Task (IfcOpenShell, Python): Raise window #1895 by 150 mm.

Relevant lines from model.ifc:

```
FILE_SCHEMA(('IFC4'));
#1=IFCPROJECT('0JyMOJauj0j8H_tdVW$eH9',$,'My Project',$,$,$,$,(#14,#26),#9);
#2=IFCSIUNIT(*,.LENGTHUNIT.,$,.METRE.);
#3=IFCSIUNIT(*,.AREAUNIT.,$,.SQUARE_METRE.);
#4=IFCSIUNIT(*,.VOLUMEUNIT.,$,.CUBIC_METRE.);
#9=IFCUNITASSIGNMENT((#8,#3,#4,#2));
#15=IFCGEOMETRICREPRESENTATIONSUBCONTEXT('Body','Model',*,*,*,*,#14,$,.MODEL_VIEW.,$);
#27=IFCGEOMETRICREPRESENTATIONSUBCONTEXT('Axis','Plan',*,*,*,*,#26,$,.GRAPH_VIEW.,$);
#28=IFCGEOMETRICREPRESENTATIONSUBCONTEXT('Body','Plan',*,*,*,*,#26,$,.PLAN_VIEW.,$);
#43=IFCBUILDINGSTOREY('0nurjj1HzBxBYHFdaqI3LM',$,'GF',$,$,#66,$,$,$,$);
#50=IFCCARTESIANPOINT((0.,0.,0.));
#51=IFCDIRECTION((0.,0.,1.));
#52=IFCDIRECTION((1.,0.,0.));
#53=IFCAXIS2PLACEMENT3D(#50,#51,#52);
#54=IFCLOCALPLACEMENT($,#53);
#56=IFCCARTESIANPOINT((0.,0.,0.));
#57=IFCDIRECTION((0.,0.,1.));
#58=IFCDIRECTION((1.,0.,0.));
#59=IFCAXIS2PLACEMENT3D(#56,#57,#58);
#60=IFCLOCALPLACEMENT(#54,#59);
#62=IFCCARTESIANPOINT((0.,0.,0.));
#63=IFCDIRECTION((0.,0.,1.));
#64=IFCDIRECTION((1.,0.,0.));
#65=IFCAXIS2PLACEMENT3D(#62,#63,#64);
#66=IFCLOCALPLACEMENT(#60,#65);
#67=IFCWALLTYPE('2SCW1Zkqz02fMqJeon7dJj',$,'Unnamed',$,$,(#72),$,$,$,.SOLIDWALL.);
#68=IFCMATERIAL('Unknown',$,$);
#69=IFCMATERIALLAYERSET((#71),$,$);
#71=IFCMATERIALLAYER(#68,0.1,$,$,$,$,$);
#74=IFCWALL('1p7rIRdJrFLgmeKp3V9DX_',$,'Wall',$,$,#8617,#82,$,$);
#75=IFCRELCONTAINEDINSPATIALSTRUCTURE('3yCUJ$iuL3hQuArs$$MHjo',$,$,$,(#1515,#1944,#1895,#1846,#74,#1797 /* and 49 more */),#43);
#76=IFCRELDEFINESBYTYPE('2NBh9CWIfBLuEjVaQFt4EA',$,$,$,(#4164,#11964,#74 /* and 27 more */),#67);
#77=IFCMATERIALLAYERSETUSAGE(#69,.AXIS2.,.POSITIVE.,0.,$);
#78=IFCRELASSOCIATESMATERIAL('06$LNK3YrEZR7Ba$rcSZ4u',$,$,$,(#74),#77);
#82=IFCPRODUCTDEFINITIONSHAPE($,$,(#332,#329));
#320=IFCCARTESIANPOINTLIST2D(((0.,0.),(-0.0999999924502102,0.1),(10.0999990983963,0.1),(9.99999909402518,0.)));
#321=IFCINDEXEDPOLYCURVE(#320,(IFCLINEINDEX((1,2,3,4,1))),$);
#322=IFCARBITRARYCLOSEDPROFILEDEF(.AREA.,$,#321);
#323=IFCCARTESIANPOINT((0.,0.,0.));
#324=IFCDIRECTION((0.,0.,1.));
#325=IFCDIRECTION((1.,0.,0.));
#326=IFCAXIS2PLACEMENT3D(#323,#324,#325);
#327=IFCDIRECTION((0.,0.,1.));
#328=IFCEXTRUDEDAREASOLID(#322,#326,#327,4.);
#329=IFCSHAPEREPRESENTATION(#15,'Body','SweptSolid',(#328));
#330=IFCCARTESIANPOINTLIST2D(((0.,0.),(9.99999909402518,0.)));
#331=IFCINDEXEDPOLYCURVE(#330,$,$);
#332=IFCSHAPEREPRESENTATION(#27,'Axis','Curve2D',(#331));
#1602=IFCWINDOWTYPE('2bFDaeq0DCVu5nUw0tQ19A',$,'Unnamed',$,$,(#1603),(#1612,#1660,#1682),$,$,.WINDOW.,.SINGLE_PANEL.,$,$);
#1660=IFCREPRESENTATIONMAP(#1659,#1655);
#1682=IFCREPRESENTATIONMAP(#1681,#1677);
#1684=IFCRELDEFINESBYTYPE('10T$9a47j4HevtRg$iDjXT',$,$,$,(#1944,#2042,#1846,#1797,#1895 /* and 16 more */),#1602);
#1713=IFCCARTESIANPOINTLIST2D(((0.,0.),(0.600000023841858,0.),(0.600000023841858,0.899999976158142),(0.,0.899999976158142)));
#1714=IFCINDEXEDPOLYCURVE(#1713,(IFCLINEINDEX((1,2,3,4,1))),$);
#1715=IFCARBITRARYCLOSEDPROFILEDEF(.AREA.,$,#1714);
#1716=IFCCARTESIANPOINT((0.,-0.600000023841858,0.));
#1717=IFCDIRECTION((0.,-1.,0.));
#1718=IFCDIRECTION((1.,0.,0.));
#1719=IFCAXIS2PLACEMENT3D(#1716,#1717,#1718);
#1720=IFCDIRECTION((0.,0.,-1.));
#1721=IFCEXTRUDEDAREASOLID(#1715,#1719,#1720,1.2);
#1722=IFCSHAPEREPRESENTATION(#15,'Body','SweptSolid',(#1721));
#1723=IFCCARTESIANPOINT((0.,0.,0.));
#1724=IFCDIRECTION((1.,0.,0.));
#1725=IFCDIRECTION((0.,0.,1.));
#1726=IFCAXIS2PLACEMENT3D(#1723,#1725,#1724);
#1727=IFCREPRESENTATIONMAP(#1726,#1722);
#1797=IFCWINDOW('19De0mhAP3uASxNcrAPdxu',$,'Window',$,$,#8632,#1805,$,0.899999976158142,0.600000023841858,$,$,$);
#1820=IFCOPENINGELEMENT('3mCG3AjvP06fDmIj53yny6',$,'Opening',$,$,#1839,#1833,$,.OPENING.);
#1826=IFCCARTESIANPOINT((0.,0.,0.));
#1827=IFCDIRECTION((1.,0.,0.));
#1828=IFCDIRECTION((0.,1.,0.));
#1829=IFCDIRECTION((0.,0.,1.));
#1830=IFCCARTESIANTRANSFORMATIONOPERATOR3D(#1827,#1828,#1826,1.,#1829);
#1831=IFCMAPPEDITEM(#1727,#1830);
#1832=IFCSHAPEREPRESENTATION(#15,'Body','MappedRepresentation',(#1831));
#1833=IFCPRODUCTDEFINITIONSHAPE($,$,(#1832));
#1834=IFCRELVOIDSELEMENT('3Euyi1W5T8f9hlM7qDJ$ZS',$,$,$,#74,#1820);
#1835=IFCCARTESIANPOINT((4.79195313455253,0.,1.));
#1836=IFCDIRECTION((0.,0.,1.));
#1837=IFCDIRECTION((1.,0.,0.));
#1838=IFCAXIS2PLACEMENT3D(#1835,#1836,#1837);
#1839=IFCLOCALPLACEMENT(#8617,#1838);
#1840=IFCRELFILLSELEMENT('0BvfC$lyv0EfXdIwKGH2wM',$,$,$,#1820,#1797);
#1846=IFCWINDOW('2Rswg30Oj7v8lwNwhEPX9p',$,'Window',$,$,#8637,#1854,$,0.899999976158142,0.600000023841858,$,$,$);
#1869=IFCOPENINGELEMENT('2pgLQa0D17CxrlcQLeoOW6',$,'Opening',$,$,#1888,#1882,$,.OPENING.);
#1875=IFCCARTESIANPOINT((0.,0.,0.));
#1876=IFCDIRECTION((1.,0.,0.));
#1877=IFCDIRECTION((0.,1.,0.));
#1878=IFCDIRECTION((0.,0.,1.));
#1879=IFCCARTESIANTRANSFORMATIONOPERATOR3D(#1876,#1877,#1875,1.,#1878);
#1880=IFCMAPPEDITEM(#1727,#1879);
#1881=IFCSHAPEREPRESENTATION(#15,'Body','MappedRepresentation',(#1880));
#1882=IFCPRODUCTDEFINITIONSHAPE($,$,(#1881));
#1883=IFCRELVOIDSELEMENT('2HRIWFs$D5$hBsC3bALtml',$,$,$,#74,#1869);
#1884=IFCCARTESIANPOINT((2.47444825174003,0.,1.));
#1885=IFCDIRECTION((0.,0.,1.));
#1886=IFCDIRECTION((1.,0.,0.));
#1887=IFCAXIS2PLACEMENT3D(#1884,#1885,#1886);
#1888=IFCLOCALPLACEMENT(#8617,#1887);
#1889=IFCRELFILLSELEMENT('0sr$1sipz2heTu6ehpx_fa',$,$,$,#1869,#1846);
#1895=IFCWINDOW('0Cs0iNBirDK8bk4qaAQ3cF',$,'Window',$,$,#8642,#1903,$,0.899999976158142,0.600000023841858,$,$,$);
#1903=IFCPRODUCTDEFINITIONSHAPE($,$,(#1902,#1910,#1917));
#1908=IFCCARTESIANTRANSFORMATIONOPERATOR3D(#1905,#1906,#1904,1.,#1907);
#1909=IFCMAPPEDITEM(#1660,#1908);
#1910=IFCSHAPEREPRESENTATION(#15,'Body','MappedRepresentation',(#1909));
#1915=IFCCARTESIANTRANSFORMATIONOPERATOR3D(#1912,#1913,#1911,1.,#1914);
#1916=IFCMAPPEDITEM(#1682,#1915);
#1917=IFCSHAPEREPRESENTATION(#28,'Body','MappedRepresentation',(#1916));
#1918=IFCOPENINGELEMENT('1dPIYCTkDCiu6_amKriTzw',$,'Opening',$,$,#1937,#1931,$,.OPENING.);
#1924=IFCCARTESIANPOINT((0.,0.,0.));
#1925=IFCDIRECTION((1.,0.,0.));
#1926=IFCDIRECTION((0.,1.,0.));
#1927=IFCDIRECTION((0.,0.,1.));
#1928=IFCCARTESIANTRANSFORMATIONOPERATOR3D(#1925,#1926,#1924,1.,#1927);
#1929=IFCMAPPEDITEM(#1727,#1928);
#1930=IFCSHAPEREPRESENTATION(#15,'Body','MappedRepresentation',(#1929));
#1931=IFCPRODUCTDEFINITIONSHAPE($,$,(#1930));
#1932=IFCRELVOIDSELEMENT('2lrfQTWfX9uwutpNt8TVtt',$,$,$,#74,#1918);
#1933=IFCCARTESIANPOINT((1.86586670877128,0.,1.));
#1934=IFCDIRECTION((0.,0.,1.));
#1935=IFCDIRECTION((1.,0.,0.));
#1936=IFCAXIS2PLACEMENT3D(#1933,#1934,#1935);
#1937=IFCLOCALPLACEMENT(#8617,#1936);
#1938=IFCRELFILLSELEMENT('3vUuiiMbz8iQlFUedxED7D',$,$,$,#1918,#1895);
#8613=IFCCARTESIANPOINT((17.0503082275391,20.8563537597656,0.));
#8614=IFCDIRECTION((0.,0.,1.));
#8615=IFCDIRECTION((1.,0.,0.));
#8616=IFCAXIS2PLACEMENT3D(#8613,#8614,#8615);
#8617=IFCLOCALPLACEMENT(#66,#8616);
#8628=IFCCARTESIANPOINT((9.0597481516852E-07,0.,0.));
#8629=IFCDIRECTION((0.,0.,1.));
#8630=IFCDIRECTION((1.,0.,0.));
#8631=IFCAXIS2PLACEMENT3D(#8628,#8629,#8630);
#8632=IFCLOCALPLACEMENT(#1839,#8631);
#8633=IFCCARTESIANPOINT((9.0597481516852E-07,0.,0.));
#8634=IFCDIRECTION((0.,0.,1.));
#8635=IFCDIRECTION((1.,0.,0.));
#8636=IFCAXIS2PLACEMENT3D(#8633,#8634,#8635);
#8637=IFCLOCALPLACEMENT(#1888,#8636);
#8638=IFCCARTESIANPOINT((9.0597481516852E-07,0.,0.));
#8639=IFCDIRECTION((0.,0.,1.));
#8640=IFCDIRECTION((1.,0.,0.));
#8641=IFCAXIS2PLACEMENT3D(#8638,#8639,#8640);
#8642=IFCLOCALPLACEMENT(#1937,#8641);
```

```python
import numpy as np
import ifcopenshell
import ifcopenshell.api.geometry
import ifcopenshell.util.placement
import ifcopenshell.util.unit

model = ifcopenshell.open("model.ifc")
unit_scale = ifcopenshell.util.unit.calculate_unit_scale(model)

window = model.by_guid("0Cs0iNBirDK8bk4qaAQ3cF")
opening = window.FillsVoids[0].RelatingOpeningElement
dz = 0.15 / unit_scale

shift = np.array([0.0, 0.0, dz])
# The window is placed relative to its opening, so it follows when the opening moves.
matrix = ifcopenshell.util.placement.get_local_placement(opening.ObjectPlacement)
matrix[:3, 3] += shift
ifcopenshell.api.geometry.edit_object_placement(
    model, product=opening, matrix=matrix, is_si=False, should_transform_children=True
)

print(f"moved by {dz * unit_scale:+.3f} m")

model.write("model_edited.ifc")
```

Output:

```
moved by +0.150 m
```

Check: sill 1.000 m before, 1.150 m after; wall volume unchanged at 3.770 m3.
